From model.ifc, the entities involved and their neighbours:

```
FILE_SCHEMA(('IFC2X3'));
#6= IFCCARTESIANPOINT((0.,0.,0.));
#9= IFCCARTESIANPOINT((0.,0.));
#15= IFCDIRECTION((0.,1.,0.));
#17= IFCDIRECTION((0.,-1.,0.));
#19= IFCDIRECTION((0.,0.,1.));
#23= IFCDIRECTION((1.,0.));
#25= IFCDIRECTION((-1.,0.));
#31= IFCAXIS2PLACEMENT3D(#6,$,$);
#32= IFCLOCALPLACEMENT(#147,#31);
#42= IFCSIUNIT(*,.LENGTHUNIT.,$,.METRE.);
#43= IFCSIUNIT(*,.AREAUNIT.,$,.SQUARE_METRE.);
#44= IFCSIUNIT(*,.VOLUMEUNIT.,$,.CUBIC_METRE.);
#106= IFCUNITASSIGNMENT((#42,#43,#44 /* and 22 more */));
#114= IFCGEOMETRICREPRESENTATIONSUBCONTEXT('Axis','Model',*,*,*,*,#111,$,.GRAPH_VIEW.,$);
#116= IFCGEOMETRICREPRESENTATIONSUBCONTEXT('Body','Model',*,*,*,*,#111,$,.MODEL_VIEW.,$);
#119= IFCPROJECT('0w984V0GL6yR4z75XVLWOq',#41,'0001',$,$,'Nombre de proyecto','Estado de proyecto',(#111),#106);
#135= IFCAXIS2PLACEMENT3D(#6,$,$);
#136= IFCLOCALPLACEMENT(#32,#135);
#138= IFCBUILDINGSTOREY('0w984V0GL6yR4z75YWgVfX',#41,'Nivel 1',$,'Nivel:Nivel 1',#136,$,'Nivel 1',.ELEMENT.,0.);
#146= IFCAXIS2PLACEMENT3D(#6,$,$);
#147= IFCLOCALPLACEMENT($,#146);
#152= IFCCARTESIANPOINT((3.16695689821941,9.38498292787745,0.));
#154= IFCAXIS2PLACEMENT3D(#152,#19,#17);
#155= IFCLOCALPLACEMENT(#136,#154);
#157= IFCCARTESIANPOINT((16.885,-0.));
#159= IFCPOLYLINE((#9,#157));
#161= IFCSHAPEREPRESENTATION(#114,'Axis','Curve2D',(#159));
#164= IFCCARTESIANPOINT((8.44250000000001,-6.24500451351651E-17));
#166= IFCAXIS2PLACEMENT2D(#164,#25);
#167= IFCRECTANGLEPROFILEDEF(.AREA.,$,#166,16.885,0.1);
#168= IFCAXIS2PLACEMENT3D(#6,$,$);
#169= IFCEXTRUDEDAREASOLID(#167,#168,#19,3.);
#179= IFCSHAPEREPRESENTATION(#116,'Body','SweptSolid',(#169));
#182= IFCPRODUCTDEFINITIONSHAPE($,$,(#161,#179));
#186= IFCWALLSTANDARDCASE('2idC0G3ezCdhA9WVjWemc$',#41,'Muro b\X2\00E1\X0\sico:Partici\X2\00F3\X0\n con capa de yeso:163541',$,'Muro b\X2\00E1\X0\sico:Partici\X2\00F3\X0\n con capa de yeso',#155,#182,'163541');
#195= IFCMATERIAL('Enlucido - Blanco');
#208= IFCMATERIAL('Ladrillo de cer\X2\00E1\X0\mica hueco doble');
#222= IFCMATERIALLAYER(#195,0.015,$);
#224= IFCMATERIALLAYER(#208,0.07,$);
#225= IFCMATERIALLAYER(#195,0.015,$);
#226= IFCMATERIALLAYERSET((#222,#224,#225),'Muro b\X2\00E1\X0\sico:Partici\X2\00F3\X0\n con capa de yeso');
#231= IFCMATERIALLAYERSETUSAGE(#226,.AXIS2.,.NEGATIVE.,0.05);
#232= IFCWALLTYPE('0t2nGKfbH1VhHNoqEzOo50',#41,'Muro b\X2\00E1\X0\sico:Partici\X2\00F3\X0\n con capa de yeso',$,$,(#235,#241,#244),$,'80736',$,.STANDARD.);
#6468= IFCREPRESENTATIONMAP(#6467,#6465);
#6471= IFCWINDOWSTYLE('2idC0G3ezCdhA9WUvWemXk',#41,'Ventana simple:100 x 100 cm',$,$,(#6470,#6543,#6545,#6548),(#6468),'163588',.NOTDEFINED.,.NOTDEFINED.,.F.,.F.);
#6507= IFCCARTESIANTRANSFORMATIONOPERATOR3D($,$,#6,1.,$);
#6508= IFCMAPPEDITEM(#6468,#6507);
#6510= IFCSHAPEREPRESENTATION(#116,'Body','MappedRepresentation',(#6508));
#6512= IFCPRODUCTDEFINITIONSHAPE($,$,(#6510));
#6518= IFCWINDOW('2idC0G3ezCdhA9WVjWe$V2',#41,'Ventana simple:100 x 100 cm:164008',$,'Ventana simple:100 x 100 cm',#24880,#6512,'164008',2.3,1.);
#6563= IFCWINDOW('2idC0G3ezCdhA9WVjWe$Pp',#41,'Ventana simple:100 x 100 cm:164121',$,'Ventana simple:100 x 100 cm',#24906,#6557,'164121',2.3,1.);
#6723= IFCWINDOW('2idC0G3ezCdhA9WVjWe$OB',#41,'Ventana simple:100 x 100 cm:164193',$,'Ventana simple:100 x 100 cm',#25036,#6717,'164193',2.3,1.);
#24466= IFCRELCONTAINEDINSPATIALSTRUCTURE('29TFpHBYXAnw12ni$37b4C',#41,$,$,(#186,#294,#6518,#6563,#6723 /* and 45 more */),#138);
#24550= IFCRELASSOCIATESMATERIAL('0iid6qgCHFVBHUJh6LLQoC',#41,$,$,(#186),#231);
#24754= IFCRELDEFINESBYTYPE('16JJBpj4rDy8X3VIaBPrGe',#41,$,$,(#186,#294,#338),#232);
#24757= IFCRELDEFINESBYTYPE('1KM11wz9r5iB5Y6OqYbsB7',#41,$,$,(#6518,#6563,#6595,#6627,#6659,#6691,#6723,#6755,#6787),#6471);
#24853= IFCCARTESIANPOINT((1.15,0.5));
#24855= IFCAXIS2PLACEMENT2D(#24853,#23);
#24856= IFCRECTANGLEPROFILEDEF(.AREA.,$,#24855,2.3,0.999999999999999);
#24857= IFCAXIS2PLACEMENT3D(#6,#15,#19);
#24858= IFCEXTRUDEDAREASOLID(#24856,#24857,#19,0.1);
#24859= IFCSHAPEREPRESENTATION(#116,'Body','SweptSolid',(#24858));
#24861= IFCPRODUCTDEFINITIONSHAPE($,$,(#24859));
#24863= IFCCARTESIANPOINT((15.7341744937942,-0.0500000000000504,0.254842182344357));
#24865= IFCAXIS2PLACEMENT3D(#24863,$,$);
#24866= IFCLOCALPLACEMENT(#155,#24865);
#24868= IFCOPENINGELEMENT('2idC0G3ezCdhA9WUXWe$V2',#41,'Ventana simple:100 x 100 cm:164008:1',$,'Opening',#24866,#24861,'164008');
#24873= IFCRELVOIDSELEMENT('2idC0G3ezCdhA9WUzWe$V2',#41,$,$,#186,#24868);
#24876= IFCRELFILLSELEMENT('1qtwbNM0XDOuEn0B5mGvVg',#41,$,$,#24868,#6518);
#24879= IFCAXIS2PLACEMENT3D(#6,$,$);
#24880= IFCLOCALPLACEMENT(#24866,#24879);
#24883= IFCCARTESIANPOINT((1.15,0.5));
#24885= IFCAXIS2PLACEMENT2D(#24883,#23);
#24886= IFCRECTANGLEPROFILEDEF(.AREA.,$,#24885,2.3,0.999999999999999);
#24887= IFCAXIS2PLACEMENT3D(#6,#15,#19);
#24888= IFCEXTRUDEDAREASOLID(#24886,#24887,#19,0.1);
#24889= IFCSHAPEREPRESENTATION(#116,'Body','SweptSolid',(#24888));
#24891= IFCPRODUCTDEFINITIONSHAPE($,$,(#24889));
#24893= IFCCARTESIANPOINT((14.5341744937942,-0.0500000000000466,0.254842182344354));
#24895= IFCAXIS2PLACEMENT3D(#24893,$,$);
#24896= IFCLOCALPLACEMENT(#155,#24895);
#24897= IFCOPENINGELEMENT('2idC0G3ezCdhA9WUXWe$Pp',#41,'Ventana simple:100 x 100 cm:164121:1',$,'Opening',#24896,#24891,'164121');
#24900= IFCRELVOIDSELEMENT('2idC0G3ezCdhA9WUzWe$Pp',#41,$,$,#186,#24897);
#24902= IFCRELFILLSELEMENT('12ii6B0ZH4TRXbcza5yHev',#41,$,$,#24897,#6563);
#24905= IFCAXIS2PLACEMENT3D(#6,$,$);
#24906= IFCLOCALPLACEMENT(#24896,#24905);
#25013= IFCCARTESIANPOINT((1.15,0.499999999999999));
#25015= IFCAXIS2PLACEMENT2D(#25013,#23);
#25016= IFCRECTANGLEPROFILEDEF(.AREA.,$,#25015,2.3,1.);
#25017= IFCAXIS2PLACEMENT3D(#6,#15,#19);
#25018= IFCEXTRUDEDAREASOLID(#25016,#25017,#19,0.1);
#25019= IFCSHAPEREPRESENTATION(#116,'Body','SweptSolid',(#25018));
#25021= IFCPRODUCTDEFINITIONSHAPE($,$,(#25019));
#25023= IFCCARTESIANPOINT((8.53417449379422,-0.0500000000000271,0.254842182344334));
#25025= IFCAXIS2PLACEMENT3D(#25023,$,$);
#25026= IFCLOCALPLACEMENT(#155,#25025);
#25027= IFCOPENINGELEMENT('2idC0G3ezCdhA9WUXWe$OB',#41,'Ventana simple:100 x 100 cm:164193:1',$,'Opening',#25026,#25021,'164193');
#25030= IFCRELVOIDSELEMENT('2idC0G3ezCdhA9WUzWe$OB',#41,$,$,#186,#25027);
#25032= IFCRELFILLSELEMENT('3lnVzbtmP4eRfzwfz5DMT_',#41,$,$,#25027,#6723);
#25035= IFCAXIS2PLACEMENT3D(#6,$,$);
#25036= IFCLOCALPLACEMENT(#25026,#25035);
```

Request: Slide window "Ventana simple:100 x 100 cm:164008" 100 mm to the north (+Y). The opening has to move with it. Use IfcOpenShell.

```python
import ifcopenshell
import ifcopenshell.api.geometry
import ifcopenshell.util.placement

model = ifcopenshell.open("model.ifc")

window = model.by_guid("2idC0G3ezCdhA9WVjWe$V2")
opening = window.FillsVoids[0].RelatingOpeningElement
wall = opening.VoidsElements[0].RelatingBuildingElement

wall_matrix = ifcopenshell.util.placement.get_local_placement(wall.ObjectPlacement)
shift = wall_matrix[:3, 0] * -0.1
before = ifcopenshell.util.placement.get_local_placement(window.ObjectPlacement)[:3, 3].copy()

# The window is placed relative to its opening, so it follows when the opening moves.
matrix = ifcopenshell.util.placement.get_local_placement(opening.ObjectPlacement)
matrix[:3, 3] += shift
ifcopenshell.api.geometry.edit_object_placement(
    model, product=opening, matrix=matrix, is_si=False, should_transform_children=True
)

after = ifcopenshell.util.placement.get_local_placement(window.ObjectPlacement)[:3, 3]
print("window moved by", (after - before).round(3) + 0.0)

model.write("model_v2.ifc")
```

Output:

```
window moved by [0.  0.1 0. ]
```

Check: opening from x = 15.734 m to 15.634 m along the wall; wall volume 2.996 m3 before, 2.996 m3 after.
